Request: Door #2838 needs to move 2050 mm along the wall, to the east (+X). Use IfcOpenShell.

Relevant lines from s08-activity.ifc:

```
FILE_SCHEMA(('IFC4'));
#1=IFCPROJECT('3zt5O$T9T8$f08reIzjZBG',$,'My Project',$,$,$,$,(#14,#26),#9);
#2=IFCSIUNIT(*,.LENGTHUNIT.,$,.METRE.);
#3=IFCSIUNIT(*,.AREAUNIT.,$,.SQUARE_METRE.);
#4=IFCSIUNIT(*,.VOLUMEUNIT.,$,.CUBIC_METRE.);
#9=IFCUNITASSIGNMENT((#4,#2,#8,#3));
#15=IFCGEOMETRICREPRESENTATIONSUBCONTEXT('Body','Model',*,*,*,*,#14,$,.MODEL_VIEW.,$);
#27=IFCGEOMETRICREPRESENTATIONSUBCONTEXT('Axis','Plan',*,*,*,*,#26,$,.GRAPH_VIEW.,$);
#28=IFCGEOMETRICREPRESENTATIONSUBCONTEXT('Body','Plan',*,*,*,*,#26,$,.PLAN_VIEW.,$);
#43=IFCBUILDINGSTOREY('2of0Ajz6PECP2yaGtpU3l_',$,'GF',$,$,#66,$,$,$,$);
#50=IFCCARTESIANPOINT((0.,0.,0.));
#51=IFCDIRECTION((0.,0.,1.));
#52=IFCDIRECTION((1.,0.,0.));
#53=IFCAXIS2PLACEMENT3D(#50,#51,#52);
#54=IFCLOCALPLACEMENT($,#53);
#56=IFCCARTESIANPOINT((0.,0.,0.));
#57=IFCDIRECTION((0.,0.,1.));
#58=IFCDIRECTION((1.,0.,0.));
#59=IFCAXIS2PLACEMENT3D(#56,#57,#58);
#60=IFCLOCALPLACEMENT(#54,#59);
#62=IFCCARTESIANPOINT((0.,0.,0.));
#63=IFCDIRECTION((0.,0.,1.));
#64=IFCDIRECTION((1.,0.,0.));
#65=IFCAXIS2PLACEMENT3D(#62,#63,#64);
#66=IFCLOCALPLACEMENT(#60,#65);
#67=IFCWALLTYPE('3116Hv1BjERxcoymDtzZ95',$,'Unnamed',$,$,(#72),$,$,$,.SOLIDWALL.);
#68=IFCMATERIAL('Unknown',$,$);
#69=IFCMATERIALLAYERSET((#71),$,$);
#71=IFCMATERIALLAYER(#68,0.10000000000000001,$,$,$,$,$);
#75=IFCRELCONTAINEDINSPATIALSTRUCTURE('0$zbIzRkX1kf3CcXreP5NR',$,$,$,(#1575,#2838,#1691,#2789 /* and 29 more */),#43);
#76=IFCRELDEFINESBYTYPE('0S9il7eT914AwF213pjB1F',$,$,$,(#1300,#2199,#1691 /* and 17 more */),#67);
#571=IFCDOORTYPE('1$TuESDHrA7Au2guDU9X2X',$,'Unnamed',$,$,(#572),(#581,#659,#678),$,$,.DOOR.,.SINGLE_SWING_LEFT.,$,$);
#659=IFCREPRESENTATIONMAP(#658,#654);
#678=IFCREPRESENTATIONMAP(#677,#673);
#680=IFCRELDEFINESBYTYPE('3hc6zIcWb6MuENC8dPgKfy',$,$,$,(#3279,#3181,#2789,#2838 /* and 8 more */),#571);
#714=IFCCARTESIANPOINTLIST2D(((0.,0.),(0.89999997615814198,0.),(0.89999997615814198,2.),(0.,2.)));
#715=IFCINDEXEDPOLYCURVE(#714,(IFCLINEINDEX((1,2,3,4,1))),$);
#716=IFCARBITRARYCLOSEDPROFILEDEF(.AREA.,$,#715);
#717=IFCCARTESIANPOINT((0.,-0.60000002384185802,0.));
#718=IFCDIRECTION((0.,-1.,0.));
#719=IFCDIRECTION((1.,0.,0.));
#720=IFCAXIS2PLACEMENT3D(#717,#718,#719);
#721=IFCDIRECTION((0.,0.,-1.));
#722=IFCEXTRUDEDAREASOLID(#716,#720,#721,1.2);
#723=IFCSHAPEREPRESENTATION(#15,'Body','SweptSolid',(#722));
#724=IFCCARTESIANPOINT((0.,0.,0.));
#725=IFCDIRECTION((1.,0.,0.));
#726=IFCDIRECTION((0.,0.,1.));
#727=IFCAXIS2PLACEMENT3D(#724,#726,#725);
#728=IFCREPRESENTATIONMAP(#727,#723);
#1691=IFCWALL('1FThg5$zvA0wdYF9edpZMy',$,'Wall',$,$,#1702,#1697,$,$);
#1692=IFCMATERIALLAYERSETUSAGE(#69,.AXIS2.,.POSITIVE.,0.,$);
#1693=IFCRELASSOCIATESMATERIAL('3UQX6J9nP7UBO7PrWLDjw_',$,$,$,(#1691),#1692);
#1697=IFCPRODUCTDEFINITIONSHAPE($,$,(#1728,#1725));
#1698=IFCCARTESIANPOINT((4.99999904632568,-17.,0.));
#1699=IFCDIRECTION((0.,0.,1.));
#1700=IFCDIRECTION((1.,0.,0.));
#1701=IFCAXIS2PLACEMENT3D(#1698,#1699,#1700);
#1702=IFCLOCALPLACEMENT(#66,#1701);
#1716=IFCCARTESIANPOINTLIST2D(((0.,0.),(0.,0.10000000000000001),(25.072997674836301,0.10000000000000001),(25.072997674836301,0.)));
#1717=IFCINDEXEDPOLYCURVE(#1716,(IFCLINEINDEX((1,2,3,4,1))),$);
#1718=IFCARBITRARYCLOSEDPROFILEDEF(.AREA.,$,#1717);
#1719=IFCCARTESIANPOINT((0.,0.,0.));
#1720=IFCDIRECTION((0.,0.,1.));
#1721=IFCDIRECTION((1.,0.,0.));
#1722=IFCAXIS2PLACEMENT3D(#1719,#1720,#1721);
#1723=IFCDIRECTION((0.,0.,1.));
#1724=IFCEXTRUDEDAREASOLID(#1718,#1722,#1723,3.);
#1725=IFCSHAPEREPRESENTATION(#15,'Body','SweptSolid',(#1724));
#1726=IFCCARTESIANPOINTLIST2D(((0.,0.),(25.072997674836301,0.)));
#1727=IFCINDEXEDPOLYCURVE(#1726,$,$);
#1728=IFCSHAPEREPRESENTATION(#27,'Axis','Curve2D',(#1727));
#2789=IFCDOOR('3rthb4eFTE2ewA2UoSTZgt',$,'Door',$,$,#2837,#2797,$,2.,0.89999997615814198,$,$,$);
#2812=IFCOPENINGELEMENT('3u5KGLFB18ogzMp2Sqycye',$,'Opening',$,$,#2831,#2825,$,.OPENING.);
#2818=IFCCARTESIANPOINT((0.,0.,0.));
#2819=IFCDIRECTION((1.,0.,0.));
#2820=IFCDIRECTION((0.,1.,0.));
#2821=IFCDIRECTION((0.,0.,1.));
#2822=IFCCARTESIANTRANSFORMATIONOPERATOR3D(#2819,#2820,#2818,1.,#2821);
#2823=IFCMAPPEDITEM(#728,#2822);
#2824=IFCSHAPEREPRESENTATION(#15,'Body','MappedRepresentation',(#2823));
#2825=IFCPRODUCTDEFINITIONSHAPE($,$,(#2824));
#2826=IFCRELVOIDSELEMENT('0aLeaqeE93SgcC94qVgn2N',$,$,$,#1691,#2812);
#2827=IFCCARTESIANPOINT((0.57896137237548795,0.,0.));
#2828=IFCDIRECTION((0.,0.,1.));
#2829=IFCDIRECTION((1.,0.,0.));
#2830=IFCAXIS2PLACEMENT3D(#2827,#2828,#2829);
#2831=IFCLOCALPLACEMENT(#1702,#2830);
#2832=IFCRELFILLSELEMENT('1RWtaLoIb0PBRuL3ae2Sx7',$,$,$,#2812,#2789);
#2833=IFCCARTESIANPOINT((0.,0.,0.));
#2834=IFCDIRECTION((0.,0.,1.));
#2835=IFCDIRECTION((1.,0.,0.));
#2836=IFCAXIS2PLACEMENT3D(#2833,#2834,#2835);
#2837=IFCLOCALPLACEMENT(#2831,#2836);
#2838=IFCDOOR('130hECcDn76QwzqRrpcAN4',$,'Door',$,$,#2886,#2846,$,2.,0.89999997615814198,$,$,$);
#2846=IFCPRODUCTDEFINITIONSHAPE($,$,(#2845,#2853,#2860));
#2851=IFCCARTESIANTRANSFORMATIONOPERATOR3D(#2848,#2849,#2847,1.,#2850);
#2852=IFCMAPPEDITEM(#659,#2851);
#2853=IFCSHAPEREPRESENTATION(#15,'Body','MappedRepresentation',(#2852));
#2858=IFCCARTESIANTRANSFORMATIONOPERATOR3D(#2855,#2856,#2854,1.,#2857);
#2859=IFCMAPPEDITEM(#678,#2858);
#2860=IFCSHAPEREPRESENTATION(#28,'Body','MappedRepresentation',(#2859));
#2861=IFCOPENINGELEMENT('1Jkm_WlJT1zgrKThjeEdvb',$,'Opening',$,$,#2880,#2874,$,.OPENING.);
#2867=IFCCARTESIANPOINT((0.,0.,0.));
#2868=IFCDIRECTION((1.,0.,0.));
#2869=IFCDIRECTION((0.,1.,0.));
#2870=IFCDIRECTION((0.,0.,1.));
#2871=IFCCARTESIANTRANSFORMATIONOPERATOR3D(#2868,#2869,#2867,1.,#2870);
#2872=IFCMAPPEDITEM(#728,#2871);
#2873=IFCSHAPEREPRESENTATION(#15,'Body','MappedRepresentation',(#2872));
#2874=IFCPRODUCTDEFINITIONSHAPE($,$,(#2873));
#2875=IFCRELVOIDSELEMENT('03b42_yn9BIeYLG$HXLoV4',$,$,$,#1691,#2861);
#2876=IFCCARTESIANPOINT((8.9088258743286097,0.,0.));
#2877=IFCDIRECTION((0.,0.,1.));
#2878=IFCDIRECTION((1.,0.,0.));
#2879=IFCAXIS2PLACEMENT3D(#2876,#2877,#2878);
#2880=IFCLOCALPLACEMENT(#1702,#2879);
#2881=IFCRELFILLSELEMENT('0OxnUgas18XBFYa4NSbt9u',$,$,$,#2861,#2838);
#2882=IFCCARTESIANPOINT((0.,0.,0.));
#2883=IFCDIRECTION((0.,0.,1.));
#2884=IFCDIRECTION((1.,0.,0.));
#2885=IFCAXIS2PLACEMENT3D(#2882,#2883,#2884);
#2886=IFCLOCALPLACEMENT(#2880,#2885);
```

```python
import ifcopenshell
import ifcopenshell.api.geometry
import ifcopenshell.util.placement
import ifcopenshell.util.unit

model = ifcopenshell.open("s08-activity.ifc")
unit_scale = ifcopenshell.util.unit.calculate_unit_scale(model)

door = model.by_guid("130hECcDn76QwzqRrpcAN4")
opening = door.FillsVoids[0].RelatingOpeningElement
wall = opening.VoidsElements[0].RelatingBuildingElement

wall_matrix = ifcopenshell.util.placement.get_local_placement(wall.ObjectPlacement)
shift = wall_matrix[:3, 0] * 2.05 / unit_scale
before = ifcopenshell.util.placement.get_local_placement(door.ObjectPlacement)[:3, 3].copy()

# The door is placed relative to its opening, so it follows when the opening moves.
matrix = ifcopenshell.util.placement.get_local_placement(opening.ObjectPlacement)
matrix[:3, 3] += shift
ifcopenshell.api.geometry.edit_object_placement(
    model, product=opening, matrix=matrix, is_si=False, should_transform_children=True
)

after = ifcopenshell.util.placement.get_local_placement(door.ObjectPlacement)[:3, 3]
print("door moved by", (after - before).round(3) + 0.0)

model.write("s08-activity_rev.ifc")
```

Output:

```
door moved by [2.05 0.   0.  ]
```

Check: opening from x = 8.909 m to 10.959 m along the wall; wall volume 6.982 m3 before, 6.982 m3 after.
